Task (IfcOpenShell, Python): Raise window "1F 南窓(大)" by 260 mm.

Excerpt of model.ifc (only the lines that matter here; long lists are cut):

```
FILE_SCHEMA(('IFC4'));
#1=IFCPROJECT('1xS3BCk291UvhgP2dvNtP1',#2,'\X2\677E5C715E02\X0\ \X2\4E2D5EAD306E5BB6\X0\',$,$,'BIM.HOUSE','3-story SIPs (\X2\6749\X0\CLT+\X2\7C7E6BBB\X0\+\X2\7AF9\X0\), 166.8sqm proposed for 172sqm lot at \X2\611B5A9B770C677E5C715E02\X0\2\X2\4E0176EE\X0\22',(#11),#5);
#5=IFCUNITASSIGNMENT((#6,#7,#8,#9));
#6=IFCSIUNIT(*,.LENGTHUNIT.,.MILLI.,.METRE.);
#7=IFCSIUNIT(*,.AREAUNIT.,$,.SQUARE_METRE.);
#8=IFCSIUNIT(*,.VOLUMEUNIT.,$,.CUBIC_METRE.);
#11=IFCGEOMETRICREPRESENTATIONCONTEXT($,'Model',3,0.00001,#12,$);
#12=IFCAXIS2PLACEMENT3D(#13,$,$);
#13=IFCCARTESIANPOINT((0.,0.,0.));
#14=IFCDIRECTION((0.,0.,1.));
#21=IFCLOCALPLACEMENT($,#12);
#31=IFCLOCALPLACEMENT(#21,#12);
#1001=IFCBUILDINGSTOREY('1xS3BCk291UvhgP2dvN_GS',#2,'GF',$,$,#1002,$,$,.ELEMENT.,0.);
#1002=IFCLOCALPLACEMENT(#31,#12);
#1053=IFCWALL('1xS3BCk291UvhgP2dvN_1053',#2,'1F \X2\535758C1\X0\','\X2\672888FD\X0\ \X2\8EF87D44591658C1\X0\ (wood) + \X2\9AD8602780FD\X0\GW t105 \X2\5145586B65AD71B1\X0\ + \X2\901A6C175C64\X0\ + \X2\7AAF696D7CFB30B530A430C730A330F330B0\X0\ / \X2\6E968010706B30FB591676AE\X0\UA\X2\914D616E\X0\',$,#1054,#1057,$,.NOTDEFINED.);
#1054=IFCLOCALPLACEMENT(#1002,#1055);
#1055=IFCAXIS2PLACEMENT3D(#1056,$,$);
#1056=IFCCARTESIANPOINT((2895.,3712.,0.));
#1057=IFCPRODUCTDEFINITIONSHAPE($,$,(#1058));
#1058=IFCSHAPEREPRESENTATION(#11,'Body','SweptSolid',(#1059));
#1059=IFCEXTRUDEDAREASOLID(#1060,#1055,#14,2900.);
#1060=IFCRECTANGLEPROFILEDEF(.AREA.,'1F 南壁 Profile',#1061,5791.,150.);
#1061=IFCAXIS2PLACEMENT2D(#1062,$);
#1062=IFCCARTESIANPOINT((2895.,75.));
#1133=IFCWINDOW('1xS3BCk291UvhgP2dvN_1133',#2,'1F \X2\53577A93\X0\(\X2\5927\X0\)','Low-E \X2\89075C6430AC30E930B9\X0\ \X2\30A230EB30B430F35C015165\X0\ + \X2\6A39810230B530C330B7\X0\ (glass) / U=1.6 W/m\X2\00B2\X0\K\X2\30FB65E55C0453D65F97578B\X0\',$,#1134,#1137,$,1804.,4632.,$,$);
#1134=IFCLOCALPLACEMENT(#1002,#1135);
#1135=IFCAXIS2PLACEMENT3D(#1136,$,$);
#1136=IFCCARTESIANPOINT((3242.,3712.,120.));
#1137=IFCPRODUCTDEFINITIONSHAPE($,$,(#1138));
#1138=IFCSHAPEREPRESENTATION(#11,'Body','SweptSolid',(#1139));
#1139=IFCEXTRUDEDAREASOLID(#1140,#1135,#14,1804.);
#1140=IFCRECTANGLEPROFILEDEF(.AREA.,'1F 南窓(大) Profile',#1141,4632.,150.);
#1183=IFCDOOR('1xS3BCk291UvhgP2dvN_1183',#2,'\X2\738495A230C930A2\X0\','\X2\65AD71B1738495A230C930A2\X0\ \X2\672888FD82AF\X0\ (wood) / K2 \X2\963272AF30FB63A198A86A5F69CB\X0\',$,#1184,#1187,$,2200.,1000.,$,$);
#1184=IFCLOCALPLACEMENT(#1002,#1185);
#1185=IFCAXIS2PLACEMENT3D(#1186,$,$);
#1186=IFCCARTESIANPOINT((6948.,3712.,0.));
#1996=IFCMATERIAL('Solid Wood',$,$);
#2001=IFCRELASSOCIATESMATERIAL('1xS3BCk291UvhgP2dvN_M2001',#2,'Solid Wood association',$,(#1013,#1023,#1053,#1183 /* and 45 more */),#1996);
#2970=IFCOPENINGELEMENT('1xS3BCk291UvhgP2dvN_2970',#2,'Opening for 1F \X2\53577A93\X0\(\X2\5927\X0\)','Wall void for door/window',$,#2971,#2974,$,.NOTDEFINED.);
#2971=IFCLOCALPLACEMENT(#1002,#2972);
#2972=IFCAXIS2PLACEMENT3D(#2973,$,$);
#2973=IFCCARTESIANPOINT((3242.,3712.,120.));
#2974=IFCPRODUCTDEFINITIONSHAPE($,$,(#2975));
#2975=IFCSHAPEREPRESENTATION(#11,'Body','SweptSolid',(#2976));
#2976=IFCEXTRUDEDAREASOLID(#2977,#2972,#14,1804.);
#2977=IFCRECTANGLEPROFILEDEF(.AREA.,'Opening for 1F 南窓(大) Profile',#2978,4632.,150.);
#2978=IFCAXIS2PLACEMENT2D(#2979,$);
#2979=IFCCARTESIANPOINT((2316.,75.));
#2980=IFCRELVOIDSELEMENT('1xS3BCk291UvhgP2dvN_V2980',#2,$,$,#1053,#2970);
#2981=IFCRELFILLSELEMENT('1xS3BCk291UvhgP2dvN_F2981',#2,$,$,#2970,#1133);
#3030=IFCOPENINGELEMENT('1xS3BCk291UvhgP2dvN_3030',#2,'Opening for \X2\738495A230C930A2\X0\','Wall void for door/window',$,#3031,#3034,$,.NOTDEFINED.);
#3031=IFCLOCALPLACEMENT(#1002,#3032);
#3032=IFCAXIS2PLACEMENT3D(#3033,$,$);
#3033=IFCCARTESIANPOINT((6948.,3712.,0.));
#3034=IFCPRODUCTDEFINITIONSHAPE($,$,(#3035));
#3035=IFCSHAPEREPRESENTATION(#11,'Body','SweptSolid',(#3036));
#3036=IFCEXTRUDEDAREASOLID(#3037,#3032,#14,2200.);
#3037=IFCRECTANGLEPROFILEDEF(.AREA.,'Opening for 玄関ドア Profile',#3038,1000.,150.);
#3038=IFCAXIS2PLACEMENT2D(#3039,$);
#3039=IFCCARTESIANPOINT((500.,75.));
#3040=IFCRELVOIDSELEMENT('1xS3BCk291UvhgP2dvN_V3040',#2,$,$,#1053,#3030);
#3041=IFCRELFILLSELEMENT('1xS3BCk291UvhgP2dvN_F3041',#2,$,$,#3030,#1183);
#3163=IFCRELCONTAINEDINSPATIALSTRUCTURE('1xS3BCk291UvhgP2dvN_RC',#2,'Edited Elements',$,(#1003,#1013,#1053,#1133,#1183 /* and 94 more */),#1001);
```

```python
import numpy as np
import ifcopenshell
import ifcopenshell.api.geometry
import ifcopenshell.util.placement
import ifcopenshell.util.unit

model = ifcopenshell.open("model.ifc")
unit_scale = ifcopenshell.util.unit.calculate_unit_scale(model)

window = model.by_guid("1xS3BCk291UvhgP2dvN_1133")
opening = window.FillsVoids[0].RelatingOpeningElement
dz = 0.26 / unit_scale

shift = np.array([0.0, 0.0, dz])
# The window is not placed relative to its opening, so move both.
for product in (opening, window):
    matrix = ifcopenshell.util.placement.get_local_placement(product.ObjectPlacement)
    matrix[:3, 3] += shift
    ifcopenshell.api.geometry.edit_object_placement(model, product=product, matrix=matrix, is_si=False)

print(f"moved by {dz * unit_scale:+.3f} m")

model.write("model_updated.ifc")
```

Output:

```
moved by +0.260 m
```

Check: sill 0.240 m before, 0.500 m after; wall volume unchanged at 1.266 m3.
